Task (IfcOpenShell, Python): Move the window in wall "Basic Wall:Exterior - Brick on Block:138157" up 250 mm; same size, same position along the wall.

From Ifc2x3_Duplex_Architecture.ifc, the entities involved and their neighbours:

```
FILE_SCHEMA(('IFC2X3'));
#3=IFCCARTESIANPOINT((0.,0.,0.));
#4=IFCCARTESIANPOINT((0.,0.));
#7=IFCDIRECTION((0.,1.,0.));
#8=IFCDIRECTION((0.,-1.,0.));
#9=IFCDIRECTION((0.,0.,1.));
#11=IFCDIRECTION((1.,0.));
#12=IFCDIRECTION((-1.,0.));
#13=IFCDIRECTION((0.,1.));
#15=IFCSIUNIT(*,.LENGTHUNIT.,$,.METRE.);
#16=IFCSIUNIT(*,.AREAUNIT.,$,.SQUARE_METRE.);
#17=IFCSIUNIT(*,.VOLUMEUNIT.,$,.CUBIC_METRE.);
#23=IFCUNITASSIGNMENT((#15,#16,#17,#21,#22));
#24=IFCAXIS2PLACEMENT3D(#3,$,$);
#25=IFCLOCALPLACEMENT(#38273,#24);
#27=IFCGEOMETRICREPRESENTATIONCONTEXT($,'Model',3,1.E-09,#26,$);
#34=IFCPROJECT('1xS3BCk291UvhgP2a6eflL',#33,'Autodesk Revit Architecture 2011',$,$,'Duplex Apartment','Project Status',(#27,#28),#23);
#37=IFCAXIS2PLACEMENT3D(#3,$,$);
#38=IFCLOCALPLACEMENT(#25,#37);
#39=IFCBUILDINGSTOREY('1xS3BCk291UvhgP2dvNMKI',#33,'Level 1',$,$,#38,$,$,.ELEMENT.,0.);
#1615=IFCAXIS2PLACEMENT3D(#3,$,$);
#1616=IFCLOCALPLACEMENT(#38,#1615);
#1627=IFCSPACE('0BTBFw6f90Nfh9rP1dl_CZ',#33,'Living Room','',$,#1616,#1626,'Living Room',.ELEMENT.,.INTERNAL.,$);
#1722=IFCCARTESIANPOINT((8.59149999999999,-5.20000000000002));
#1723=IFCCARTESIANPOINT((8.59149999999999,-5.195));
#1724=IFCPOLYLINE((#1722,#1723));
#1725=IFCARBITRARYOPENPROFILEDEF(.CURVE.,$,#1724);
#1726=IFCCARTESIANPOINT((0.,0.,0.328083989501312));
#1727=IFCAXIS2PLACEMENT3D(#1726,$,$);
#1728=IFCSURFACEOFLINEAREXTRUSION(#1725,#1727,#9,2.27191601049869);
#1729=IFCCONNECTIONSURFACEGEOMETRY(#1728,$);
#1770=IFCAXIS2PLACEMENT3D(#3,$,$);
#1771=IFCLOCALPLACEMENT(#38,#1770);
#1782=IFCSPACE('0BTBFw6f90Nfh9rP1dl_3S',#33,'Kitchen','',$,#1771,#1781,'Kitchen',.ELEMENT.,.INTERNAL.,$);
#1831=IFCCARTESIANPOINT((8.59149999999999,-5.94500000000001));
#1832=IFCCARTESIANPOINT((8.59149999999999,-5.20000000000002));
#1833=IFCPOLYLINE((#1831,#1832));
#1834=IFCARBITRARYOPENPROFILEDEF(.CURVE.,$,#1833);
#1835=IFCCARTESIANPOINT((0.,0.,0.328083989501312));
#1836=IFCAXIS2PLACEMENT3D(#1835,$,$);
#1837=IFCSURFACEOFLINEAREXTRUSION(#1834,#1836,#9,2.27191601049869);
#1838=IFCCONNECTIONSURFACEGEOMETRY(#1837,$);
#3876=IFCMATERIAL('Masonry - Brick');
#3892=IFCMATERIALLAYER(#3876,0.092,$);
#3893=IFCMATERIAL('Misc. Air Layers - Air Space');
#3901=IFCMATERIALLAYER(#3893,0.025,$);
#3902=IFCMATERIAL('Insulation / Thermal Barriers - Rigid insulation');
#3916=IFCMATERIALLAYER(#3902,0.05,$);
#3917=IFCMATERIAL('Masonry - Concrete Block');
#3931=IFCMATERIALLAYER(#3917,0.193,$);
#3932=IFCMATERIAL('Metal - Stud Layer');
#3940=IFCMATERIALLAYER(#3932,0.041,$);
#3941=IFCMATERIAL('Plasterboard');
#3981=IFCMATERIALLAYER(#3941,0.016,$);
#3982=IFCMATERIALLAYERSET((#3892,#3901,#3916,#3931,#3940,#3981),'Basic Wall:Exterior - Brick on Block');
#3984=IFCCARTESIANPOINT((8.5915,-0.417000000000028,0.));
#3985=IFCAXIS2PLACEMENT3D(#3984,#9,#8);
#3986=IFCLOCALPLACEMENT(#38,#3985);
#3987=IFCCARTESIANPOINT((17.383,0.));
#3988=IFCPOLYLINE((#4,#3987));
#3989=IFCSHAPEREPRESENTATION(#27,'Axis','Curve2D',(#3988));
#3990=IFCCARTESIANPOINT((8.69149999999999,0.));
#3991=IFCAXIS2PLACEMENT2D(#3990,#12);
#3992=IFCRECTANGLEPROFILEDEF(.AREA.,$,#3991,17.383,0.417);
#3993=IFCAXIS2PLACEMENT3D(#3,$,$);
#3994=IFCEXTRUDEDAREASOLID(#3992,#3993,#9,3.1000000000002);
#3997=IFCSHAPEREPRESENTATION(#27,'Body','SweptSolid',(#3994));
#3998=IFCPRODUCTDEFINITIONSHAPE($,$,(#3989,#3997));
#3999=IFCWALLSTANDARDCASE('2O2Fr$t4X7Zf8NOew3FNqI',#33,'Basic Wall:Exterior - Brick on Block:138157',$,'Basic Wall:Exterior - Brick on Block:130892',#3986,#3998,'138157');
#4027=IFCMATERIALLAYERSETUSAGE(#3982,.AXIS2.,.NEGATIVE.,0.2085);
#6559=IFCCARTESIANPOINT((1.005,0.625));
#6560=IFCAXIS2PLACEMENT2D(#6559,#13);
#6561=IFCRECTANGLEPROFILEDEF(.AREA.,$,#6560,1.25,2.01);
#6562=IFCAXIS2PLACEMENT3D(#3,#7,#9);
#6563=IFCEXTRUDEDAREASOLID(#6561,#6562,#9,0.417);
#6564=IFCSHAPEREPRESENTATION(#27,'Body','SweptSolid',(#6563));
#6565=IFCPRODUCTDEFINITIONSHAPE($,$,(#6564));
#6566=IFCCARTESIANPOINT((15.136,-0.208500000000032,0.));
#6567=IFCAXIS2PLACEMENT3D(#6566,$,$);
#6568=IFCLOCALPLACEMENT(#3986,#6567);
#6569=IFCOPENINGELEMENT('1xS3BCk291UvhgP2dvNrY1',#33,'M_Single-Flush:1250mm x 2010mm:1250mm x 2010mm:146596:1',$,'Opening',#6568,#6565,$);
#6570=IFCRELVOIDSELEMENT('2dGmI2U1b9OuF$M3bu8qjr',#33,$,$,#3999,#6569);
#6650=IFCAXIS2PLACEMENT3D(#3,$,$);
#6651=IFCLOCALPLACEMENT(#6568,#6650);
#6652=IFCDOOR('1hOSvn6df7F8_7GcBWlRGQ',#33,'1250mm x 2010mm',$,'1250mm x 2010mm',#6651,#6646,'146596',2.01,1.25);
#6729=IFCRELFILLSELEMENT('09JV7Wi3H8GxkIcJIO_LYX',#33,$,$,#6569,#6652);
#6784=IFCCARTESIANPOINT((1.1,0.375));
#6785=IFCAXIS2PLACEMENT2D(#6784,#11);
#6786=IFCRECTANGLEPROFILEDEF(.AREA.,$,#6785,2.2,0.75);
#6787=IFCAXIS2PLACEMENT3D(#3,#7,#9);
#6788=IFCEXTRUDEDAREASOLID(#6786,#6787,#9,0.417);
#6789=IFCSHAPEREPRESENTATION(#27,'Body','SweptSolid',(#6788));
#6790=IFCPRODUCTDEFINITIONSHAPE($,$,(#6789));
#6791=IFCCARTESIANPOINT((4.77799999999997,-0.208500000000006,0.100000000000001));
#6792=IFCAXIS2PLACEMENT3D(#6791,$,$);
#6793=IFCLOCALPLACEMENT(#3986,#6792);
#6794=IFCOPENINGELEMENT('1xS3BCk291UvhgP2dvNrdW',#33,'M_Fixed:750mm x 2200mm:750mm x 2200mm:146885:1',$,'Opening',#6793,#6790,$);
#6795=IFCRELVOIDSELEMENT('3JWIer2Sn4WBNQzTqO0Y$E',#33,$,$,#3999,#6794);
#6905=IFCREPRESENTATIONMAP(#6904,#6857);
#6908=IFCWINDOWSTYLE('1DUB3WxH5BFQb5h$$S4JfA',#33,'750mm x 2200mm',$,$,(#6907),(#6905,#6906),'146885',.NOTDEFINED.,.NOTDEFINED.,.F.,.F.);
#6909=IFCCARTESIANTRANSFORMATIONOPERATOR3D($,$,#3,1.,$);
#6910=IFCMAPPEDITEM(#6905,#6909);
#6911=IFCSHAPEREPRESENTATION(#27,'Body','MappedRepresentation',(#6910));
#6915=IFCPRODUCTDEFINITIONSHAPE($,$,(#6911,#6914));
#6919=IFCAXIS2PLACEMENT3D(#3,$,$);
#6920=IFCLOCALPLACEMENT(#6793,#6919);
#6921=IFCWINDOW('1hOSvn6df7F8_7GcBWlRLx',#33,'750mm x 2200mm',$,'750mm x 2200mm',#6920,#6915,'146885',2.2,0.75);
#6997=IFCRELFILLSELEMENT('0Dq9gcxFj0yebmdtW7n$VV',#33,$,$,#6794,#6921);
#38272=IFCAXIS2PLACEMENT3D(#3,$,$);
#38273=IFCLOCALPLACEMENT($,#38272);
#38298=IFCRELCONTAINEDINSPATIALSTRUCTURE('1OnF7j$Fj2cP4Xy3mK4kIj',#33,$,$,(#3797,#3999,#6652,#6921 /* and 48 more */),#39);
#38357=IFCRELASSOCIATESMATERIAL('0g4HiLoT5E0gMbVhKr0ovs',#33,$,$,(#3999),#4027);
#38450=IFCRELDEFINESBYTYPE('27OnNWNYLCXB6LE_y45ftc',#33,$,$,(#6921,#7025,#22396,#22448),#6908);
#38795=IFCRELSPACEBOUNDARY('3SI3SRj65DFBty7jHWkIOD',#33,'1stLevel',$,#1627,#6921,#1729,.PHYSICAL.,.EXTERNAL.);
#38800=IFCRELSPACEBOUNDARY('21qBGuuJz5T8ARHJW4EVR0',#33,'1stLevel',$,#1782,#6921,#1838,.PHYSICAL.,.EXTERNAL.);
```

```python
import numpy as np
import ifcopenshell
import ifcopenshell.api.geometry
import ifcopenshell.util.placement
import ifcopenshell.util.unit

model = ifcopenshell.open("Ifc2x3_Duplex_Architecture.ifc")
unit_scale = ifcopenshell.util.unit.calculate_unit_scale(model)

window = model.by_guid("1hOSvn6df7F8_7GcBWlRLx")
opening = window.FillsVoids[0].RelatingOpeningElement
dz = 0.25 / unit_scale

shift = np.array([0.0, 0.0, dz])
# The window is placed relative to its opening, so it follows when the opening moves.
matrix = ifcopenshell.util.placement.get_local_placement(opening.ObjectPlacement)
matrix[:3, 3] += shift
ifcopenshell.api.geometry.edit_object_placement(
    model, product=opening, matrix=matrix, is_si=False, should_transform_children=True
)

# Space boundary surfaces are stored in each space's coordinates; move them too.
for rel in window.ProvidesBoundaries:
    if not rel.ConnectionGeometry:
        continue
    surface = rel.ConnectionGeometry.SurfaceOnRelatingElement
    space_matrix = ifcopenshell.util.placement.get_local_placement(rel.RelatingSpace.ObjectPlacement)
    point = np.array(surface.Position.Location.Coordinates) + space_matrix[:3, :3].T @ shift
    surface.Position = model.createIfcAxis2Placement3D(
        model.createIfcCartesianPoint(point.tolist()), surface.Position.Axis, surface.Position.RefDirection
    )

print(f"moved by {dz * unit_scale:+.3f} m")

model.write("Ifc2x3_Duplex_Architecture_edited.ifc")
```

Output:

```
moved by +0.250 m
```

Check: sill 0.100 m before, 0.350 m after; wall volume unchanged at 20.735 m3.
